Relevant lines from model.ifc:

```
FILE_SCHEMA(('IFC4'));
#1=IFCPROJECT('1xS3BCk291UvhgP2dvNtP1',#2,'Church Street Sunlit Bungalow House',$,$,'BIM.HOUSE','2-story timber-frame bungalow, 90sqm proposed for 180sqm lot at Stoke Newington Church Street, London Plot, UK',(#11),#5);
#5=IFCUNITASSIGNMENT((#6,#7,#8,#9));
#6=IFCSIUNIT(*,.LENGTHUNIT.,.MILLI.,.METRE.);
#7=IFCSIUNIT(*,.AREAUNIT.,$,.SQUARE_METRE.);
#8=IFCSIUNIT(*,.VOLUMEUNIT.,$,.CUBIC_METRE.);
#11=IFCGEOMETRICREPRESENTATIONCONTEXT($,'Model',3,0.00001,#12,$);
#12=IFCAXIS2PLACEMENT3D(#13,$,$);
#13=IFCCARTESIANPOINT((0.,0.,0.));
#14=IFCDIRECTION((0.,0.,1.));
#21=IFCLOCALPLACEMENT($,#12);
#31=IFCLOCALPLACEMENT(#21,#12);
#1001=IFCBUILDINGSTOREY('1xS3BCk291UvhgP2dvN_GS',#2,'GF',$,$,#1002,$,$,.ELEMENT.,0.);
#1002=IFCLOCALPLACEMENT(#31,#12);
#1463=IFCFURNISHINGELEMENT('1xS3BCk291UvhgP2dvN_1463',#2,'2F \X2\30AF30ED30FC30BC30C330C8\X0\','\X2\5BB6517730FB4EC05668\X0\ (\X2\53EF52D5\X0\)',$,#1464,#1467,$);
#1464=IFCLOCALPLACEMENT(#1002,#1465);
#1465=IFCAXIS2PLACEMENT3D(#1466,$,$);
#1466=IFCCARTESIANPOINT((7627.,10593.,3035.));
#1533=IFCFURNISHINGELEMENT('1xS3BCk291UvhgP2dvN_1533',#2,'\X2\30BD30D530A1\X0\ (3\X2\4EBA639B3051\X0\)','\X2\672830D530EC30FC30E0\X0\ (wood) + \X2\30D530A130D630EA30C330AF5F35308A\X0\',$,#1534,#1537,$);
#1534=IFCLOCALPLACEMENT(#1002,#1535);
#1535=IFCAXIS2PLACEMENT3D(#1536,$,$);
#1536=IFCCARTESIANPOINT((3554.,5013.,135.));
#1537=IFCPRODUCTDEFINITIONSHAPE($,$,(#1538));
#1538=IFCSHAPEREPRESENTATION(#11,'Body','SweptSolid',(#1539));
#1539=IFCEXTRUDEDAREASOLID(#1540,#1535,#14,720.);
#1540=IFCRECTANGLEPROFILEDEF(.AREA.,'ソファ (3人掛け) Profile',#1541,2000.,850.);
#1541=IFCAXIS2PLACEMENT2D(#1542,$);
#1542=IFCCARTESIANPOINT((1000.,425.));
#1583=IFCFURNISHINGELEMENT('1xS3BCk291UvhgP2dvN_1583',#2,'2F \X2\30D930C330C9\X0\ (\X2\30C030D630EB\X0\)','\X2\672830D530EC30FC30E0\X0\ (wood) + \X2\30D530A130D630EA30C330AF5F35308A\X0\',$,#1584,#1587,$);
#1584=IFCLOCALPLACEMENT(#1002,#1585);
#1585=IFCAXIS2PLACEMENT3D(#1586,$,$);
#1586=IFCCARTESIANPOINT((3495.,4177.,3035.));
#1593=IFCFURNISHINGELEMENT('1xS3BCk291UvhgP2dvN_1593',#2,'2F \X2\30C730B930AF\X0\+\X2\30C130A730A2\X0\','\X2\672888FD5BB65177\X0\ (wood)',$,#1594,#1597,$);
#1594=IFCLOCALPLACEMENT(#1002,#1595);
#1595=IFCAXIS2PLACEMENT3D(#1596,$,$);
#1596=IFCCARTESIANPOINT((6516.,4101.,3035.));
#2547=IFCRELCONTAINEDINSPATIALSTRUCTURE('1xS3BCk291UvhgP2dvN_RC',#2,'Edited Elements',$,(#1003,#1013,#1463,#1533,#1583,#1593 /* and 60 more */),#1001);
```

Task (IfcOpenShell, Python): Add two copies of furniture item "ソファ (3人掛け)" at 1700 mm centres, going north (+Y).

```python
import numpy as np
import ifcopenshell
import ifcopenshell.api.geometry
import ifcopenshell.api.root
import ifcopenshell.util.element
import ifcopenshell.util.placement

model = ifcopenshell.open("model.ifc")


def reuse_history(source, copy):
    """copy_class also copies each property set's owner history, people and application; keep the originals."""
    for rel in copy.IsDefinedBy:
        if rel.is_a("IfcRelDefinesByProperties") and (history := rel.RelatingPropertyDefinition.OwnerHistory):
            rel.RelatingPropertyDefinition.OwnerHistory = source.OwnerHistory
            ifcopenshell.util.element.remove_deep2(model, history)


source = model.by_guid("1xS3BCk291UvhgP2dvN_1533")
base = ifcopenshell.util.placement.get_local_placement(source.ObjectPlacement)
step = np.array([0.0, 1.0, 0.0]) * 1700.0

for i in range(1, 3):
    copy = ifcopenshell.api.root.copy_class(model, product=source)
    copy.Representation = ifcopenshell.util.element.copy_deep(
        model, source.Representation, exclude=["IfcGeometricRepresentationContext", "IfcRepresentationMap"]
    )
    reuse_history(source, copy)
    matrix = base.copy()
    matrix[:3, 3] += i * step
    print("added at", matrix[:3, 3].round(3) + 0.0)
    ifcopenshell.api.geometry.edit_object_placement(model, product=copy, matrix=matrix, is_si=False)

model.write("model_rev.ifc")
```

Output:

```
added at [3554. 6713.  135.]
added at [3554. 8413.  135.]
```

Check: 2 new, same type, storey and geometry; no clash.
